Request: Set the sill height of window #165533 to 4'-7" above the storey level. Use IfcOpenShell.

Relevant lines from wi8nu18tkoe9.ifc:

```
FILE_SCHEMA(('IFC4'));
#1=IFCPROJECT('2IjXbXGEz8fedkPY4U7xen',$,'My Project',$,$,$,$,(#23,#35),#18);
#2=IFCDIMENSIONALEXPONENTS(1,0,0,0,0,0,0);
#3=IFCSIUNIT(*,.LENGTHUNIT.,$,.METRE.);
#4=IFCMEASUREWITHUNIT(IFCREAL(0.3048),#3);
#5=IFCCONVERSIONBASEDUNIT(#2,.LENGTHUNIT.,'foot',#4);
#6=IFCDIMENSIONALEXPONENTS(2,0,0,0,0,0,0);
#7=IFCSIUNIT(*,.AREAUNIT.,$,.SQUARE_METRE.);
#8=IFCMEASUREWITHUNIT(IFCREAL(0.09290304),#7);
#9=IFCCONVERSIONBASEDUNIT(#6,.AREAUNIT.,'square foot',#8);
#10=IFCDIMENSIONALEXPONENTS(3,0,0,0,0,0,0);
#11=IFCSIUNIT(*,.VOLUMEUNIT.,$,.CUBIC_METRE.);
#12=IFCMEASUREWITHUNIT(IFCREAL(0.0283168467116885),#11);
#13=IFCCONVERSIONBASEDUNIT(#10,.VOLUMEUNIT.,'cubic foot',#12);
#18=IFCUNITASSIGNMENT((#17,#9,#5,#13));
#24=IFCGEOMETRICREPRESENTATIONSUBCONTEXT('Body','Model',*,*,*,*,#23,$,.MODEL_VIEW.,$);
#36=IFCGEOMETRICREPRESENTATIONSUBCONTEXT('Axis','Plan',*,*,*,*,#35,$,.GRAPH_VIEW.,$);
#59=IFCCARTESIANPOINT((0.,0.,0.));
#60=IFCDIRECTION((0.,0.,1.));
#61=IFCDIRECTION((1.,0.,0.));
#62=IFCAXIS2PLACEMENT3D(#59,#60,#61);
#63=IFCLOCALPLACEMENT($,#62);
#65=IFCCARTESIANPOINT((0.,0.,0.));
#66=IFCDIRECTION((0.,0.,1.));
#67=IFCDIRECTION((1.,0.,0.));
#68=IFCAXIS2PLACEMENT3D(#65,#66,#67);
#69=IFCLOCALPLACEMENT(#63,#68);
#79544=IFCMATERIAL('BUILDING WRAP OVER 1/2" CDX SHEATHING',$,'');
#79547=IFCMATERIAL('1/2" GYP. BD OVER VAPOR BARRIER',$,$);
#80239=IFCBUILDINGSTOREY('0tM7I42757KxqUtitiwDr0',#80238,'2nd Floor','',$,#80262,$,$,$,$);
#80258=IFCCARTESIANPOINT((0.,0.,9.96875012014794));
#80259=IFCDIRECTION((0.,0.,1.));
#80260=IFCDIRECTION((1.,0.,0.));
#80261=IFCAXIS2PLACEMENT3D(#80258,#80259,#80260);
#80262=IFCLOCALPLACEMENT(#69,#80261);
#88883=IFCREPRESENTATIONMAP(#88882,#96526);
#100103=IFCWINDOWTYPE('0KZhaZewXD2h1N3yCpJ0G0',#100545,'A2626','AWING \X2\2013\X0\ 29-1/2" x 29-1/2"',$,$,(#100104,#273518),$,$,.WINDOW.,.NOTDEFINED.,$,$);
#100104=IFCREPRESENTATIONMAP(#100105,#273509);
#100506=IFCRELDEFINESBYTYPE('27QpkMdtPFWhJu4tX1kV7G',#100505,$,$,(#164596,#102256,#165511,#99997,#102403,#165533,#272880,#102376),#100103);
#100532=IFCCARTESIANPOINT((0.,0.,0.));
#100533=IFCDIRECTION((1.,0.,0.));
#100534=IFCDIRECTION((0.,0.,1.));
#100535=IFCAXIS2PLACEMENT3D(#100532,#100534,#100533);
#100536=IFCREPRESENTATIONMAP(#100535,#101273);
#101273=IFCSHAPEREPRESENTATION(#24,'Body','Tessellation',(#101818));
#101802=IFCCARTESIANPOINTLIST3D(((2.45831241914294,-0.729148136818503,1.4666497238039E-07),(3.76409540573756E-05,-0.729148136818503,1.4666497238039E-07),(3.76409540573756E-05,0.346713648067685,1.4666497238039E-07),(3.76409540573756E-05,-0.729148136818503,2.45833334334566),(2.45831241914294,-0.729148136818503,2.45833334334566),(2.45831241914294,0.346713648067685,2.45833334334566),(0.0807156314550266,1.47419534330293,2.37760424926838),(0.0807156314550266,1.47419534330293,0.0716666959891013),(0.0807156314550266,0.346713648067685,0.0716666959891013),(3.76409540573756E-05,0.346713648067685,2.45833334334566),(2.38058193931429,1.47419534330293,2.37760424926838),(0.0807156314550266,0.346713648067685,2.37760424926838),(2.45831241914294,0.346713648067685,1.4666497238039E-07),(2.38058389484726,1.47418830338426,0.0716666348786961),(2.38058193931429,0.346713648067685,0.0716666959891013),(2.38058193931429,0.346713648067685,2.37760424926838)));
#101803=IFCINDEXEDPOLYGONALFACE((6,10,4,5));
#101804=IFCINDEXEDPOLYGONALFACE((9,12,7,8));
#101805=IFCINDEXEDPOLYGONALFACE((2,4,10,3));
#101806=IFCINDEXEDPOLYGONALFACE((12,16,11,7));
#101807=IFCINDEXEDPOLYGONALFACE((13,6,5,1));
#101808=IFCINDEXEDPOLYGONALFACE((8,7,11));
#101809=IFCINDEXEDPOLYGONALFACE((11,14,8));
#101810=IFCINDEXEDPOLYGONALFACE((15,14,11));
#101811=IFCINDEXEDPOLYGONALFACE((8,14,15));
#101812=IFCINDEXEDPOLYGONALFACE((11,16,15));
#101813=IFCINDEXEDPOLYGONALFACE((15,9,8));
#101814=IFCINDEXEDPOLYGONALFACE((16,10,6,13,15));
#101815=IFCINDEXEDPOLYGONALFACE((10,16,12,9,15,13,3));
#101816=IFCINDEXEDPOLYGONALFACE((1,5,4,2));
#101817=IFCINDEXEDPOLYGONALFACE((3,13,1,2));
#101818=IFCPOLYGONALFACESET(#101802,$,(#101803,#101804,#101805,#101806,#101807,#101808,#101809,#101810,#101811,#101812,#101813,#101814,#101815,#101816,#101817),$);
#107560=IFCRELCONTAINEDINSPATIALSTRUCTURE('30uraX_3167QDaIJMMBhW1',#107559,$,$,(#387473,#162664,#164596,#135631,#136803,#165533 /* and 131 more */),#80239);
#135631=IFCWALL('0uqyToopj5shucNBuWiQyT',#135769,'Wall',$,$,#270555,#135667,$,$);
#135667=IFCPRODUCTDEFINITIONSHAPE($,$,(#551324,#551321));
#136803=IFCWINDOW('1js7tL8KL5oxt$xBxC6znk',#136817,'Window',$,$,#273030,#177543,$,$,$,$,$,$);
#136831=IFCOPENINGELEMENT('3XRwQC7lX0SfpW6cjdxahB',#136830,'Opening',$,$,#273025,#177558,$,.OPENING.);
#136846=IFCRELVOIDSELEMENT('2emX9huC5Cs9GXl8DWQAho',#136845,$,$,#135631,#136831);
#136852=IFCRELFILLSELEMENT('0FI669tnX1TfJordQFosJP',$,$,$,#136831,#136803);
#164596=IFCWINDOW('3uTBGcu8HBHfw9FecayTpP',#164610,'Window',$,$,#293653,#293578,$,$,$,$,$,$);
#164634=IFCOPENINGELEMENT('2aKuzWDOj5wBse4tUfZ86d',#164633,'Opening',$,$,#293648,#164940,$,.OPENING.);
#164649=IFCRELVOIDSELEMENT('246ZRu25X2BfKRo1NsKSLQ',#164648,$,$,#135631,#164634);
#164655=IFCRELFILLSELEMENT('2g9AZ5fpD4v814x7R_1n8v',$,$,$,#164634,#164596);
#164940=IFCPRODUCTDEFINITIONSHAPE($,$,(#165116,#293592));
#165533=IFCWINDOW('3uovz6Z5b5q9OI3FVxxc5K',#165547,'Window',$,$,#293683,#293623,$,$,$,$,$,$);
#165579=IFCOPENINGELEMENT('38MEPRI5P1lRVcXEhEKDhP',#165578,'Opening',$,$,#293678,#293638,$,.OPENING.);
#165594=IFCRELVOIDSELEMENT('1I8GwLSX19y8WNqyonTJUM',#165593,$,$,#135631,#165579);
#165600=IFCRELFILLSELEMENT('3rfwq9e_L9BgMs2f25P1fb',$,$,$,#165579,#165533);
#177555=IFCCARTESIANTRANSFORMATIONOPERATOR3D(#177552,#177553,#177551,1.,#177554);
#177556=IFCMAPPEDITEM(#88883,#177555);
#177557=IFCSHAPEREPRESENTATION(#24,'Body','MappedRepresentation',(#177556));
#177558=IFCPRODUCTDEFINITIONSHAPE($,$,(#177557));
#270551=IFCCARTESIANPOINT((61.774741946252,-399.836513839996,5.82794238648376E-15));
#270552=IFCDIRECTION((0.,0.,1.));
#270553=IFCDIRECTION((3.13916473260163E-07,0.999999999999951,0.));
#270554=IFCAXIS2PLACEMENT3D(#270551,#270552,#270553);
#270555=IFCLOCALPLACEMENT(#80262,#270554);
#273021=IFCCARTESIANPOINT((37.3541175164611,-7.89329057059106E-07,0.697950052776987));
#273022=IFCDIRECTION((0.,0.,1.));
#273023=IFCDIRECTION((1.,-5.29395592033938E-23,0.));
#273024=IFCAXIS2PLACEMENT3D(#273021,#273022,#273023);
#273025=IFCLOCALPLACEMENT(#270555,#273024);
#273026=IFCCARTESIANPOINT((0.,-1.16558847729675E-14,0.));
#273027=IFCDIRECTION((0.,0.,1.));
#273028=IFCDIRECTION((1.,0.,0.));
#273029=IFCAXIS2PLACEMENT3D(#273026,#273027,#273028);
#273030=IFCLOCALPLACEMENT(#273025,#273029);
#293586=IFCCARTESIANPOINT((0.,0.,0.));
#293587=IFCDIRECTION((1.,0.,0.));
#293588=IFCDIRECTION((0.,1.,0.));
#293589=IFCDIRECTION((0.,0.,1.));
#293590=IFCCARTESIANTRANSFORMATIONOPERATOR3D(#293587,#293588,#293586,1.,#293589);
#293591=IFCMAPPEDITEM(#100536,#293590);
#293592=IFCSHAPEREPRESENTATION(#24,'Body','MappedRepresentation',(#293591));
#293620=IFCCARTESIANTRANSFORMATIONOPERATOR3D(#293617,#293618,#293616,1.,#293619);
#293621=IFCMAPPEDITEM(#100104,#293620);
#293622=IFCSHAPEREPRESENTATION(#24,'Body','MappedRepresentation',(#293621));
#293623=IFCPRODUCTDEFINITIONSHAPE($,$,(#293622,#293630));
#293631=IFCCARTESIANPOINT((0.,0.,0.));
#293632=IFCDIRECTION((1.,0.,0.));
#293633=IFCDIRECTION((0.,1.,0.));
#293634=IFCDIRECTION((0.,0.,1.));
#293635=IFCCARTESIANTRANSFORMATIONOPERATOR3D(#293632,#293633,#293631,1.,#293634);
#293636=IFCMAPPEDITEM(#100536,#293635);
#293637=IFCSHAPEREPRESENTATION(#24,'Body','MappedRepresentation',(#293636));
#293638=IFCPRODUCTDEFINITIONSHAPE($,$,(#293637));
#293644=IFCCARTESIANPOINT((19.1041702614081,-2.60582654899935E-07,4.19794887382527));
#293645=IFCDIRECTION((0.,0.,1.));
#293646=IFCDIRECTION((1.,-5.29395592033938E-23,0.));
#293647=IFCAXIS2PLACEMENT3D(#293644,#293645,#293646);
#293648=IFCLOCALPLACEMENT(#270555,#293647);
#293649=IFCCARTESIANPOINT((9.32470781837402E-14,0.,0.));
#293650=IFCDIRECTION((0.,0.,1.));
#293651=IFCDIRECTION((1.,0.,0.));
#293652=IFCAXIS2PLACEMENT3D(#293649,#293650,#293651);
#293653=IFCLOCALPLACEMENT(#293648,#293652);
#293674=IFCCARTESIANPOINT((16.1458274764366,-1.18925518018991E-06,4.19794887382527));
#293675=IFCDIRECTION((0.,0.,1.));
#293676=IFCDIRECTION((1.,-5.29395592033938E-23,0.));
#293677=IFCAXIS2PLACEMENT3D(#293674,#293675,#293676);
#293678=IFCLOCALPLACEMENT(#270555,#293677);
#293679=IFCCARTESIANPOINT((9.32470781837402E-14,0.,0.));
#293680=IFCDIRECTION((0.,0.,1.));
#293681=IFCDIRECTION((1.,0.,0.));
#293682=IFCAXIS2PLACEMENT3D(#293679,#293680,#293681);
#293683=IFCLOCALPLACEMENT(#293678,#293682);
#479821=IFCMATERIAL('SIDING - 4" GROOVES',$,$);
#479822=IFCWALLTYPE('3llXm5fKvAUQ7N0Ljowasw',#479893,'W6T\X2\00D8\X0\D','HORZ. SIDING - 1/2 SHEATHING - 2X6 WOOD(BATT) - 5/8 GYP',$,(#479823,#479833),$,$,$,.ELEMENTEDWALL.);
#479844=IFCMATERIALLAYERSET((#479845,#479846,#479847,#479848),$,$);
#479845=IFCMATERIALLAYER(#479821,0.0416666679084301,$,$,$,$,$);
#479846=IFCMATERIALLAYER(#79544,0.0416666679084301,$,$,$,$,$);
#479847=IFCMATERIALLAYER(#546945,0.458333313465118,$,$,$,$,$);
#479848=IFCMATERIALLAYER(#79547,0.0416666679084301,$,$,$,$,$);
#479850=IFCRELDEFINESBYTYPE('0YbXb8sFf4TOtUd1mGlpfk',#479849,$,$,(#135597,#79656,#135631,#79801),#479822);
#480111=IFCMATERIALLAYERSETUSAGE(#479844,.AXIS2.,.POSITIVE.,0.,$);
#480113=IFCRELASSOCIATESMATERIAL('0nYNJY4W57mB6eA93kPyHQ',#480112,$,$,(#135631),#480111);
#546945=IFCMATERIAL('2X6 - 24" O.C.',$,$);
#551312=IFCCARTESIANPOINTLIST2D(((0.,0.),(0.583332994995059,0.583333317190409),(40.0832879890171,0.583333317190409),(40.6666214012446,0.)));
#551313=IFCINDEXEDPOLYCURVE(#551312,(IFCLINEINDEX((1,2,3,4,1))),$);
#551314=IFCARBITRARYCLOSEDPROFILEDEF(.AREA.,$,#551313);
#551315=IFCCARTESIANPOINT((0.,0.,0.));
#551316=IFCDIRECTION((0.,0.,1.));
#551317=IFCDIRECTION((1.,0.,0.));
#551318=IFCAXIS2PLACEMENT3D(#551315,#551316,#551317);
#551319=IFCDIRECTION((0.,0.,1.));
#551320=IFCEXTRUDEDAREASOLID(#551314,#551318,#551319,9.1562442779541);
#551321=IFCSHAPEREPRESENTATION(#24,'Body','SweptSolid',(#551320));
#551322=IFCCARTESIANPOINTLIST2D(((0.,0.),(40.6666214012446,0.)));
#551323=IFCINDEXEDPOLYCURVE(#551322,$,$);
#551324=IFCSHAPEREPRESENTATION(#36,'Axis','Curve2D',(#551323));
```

```python
import numpy as np
import ifcopenshell
import ifcopenshell.api.geometry
import ifcopenshell.geom
import ifcopenshell.util.element
import ifcopenshell.util.placement
import ifcopenshell.util.shape
import ifcopenshell.util.unit

model = ifcopenshell.open("wi8nu18tkoe9.ifc")
unit_scale = ifcopenshell.util.unit.calculate_unit_scale(model)

window = model.by_guid("3uovz6Z5b5q9OI3FVxxc5K")
opening = window.FillsVoids[0].RelatingOpeningElement
storey = ifcopenshell.util.element.get_container(window, ifc_class="IfcBuildingStorey")
level = ifcopenshell.util.placement.get_local_placement(storey.ObjectPlacement)[2, 3]

# The opening's origin need not be at the sill, so measure its lowest point.
shape = ifcopenshell.geom.create_shape(ifcopenshell.geom.settings(), opening)
bottom = ifcopenshell.util.shape.get_shape_bottom_elevation(shape, shape.geometry) / unit_scale
dz = level + 55 * 0.0254 / unit_scale - bottom

shift = np.array([0.0, 0.0, dz])
# The window is placed relative to its opening, so it follows when the opening moves.
matrix = ifcopenshell.util.placement.get_local_placement(opening.ObjectPlacement)
matrix[:3, 3] += shift
ifcopenshell.api.geometry.edit_object_placement(
    model, product=opening, matrix=matrix, is_si=False, should_transform_children=True
)

print(f"moved by {dz * unit_scale:+.3f} m")

model.write("wi8nu18tkoe9_rev.ifc")
```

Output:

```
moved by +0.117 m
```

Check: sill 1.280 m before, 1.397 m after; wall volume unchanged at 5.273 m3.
